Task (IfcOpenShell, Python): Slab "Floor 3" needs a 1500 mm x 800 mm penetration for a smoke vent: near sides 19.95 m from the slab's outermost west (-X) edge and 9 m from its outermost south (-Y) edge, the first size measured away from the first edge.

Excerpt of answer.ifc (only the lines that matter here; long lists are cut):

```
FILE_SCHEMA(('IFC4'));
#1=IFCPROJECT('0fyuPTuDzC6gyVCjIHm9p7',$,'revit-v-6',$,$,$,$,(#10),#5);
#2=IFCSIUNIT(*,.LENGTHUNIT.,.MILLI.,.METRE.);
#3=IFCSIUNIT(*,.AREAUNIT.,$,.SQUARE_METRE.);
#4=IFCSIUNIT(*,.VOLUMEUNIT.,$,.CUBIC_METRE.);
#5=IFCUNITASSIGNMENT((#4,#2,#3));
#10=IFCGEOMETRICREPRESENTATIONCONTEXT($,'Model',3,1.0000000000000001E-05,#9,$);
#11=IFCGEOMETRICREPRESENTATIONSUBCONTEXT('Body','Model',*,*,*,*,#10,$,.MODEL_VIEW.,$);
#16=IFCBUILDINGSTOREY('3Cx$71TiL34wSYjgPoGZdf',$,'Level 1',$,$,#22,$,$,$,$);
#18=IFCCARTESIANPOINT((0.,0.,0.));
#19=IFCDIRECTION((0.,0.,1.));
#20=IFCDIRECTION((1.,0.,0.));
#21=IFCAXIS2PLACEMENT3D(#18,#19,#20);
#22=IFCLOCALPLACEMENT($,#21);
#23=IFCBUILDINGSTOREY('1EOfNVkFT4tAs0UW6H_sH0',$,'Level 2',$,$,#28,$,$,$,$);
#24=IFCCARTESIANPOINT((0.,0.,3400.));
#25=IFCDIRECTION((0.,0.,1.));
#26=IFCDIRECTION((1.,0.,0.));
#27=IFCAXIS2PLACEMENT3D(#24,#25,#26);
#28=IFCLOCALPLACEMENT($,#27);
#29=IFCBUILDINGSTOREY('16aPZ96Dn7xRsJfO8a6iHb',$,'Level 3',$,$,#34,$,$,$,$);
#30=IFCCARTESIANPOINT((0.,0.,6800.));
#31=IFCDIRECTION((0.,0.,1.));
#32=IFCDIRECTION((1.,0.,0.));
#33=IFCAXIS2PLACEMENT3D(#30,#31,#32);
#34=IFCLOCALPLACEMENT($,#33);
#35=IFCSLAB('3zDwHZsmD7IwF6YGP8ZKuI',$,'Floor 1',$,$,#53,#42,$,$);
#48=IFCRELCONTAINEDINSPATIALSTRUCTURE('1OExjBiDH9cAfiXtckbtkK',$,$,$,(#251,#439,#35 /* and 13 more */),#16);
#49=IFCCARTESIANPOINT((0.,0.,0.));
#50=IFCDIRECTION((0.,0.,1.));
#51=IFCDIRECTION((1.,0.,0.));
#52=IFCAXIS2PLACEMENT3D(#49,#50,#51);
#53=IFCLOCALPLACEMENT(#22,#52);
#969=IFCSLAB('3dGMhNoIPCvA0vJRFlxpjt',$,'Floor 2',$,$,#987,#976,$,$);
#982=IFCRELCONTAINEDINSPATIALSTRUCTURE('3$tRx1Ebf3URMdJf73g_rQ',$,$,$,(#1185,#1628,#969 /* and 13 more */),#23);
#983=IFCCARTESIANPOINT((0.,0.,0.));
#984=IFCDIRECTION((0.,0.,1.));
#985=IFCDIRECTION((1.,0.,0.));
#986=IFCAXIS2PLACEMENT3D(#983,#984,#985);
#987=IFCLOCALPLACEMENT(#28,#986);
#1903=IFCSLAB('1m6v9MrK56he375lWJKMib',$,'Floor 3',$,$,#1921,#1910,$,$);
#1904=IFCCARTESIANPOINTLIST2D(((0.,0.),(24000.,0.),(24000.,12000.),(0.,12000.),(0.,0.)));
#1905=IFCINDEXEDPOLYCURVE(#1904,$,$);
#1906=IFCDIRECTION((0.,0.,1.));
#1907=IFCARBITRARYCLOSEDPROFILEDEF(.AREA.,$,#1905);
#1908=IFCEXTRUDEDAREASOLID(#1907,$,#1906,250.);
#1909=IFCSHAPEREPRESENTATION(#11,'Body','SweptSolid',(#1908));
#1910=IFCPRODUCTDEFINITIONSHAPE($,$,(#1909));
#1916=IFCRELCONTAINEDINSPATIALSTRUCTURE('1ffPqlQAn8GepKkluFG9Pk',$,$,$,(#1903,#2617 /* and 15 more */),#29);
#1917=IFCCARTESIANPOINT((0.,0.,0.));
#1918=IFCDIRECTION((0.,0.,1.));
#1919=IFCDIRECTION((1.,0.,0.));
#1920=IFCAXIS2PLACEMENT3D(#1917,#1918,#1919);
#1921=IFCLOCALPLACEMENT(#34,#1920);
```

```python
import numpy as np
import ifcopenshell
import ifcopenshell.api.feature
import ifcopenshell.api.geometry
import ifcopenshell.api.root
import ifcopenshell.geom
import ifcopenshell.util.placement
import ifcopenshell.util.representation
import ifcopenshell.util.shape
import ifcopenshell.util.unit

model = ifcopenshell.open("answer.ifc")
unit_scale = ifcopenshell.util.unit.calculate_unit_scale(model)
settings = ifcopenshell.geom.settings()


def volume(element):
    """Net volume in cubic metres, openings subtracted."""
    shape = ifcopenshell.geom.create_shape(settings, element)
    return ifcopenshell.util.shape.get_volume(shape.geometry)


slab = model.by_guid("1m6v9MrK56he375lWJKMib")
before = volume(slab)

# Extent in the slab's own axes, in metres. The edges named are its -X and -Y sides.
slab_shape = ifcopenshell.geom.create_shape(settings, slab)
vertices = ifcopenshell.util.shape.get_vertices(slab_shape.geometry)
x_min, y_min, bottom = vertices.min(axis=0)
top = vertices[:, 2].max()

opening = ifcopenshell.api.root.create_entity(model, ifc_class="IfcOpeningElement", name="Smoke vent opening", predefined_type="OPENING")
context = ifcopenshell.util.representation.get_context(model, "Model", "Body", "MODEL_VIEW")
width, depth = 1.5, 0.8
outline = [(0.0, 0.0), (width, 0.0), (width, depth), (0.0, depth), (0.0, 0.0)]
# Overshoot both faces by 50 mm so the cut is clean.
shape = ifcopenshell.api.geometry.add_slab_representation(
    model, context=context, depth=top - bottom + 0.1, polyline=outline
)
ifcopenshell.api.geometry.assign_representation(model, product=opening, representation=shape)

matrix = ifcopenshell.util.placement.get_local_placement(slab.ObjectPlacement)
matrix[:, 3] = matrix @ np.append(np.array([x_min + 19.95, y_min + 9, bottom - 0.05]) / unit_scale, 1.0)
ifcopenshell.api.geometry.edit_object_placement(model, product=opening, matrix=matrix, is_si=False)
ifcopenshell.api.feature.add_feature(model, feature=opening, element=slab)

after = volume(slab)

print(f"slab volume {before:.3f} -> {after:.3f} m3")

model.write("answer_rev.ifc")
```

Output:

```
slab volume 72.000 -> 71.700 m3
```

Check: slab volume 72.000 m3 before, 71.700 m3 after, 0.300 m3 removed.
